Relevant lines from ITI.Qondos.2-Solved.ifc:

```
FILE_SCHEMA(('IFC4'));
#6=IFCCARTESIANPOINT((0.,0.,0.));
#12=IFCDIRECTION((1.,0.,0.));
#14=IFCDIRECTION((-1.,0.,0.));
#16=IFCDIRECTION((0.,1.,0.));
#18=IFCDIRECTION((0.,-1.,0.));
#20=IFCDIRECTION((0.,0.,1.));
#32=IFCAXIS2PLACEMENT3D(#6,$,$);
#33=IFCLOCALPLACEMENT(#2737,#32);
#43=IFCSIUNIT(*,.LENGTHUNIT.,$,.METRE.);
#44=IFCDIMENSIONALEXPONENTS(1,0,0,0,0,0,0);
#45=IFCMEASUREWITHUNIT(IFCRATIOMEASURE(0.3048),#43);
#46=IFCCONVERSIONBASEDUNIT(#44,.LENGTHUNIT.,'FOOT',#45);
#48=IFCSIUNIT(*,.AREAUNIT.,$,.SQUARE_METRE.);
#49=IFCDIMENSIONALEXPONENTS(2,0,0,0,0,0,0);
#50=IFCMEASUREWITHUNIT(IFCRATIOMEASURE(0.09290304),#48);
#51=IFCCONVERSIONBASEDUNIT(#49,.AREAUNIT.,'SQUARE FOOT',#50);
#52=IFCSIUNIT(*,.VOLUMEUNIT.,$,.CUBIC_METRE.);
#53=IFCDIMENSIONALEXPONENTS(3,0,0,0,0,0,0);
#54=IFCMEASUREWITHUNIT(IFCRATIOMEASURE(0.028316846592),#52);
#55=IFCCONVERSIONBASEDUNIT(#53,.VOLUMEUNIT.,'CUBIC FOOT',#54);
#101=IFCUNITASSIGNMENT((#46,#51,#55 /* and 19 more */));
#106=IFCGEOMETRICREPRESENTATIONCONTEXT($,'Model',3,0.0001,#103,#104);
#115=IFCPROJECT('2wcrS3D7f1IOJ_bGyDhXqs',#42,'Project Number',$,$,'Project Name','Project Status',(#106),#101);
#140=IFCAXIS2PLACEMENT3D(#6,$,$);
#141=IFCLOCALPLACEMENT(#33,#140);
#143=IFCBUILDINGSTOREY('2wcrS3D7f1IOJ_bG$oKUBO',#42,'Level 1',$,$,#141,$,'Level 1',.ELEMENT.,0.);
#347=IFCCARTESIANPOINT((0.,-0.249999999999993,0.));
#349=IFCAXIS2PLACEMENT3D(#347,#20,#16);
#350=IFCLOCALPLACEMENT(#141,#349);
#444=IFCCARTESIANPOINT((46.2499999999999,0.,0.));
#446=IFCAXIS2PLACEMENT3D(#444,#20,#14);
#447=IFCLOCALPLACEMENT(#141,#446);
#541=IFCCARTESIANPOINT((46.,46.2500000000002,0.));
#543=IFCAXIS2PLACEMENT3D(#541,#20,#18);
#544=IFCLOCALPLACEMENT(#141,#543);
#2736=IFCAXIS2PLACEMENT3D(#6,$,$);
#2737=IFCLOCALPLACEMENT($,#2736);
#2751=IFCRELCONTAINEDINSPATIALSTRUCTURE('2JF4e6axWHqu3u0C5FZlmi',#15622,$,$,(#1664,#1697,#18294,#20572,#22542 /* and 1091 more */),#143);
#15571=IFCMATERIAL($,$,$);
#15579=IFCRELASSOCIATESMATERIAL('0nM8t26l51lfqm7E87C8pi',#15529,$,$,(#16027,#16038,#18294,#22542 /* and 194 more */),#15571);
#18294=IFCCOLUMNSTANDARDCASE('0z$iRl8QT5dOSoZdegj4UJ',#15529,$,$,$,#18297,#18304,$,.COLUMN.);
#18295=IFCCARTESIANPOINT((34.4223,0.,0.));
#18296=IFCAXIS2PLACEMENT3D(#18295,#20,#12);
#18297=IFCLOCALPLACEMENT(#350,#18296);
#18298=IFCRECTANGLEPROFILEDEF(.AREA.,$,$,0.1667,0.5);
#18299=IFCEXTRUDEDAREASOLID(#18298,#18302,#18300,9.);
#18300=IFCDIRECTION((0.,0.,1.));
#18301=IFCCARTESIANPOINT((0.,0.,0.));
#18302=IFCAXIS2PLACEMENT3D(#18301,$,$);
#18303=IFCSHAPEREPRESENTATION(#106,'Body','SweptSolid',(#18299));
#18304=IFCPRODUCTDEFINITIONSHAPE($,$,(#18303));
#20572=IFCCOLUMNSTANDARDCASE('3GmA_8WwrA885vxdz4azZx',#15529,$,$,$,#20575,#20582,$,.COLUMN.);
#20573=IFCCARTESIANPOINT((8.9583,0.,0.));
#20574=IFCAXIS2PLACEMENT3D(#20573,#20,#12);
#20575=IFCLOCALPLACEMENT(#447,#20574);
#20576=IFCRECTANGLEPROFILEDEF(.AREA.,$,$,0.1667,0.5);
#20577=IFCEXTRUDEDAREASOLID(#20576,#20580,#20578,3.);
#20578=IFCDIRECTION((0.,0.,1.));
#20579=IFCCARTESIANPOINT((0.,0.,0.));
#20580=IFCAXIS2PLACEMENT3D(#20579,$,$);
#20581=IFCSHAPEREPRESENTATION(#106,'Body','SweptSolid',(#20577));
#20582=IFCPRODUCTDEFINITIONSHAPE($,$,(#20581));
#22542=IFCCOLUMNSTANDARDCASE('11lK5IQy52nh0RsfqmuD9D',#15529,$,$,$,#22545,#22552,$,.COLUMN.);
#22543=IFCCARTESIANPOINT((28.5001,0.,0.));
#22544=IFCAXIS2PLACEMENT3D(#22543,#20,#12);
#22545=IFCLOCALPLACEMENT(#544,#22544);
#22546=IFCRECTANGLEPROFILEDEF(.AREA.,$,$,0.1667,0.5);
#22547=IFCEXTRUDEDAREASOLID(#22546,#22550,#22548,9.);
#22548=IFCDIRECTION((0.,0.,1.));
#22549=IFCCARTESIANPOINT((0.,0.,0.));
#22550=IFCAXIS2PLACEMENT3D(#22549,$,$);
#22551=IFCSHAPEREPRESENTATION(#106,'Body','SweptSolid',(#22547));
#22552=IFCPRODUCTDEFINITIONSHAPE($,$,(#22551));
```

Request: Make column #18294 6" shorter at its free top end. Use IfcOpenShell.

```python
import ifcopenshell
import ifcopenshell.util.unit

model = ifcopenshell.open("ITI.Qondos.2-Solved.ifc")
unit_scale = ifcopenshell.util.unit.calculate_unit_scale(model)

member = model.by_id(18294)
change = -6 * 0.0254 / unit_scale

# The extrusion runs towards the end named, so only its depth changes.
body = next(r for r in member.Representation.Representations if r.RepresentationIdentifier == "Body")
solid = body.Items[0]
old_length = solid.Depth
solid.Depth += change

print(f"length {old_length:g} -> {solid.Depth:g}")

model.write("ITI.Qondos.2-Solved_v2.ifc")
```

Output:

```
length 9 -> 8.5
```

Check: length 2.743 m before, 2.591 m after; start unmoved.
